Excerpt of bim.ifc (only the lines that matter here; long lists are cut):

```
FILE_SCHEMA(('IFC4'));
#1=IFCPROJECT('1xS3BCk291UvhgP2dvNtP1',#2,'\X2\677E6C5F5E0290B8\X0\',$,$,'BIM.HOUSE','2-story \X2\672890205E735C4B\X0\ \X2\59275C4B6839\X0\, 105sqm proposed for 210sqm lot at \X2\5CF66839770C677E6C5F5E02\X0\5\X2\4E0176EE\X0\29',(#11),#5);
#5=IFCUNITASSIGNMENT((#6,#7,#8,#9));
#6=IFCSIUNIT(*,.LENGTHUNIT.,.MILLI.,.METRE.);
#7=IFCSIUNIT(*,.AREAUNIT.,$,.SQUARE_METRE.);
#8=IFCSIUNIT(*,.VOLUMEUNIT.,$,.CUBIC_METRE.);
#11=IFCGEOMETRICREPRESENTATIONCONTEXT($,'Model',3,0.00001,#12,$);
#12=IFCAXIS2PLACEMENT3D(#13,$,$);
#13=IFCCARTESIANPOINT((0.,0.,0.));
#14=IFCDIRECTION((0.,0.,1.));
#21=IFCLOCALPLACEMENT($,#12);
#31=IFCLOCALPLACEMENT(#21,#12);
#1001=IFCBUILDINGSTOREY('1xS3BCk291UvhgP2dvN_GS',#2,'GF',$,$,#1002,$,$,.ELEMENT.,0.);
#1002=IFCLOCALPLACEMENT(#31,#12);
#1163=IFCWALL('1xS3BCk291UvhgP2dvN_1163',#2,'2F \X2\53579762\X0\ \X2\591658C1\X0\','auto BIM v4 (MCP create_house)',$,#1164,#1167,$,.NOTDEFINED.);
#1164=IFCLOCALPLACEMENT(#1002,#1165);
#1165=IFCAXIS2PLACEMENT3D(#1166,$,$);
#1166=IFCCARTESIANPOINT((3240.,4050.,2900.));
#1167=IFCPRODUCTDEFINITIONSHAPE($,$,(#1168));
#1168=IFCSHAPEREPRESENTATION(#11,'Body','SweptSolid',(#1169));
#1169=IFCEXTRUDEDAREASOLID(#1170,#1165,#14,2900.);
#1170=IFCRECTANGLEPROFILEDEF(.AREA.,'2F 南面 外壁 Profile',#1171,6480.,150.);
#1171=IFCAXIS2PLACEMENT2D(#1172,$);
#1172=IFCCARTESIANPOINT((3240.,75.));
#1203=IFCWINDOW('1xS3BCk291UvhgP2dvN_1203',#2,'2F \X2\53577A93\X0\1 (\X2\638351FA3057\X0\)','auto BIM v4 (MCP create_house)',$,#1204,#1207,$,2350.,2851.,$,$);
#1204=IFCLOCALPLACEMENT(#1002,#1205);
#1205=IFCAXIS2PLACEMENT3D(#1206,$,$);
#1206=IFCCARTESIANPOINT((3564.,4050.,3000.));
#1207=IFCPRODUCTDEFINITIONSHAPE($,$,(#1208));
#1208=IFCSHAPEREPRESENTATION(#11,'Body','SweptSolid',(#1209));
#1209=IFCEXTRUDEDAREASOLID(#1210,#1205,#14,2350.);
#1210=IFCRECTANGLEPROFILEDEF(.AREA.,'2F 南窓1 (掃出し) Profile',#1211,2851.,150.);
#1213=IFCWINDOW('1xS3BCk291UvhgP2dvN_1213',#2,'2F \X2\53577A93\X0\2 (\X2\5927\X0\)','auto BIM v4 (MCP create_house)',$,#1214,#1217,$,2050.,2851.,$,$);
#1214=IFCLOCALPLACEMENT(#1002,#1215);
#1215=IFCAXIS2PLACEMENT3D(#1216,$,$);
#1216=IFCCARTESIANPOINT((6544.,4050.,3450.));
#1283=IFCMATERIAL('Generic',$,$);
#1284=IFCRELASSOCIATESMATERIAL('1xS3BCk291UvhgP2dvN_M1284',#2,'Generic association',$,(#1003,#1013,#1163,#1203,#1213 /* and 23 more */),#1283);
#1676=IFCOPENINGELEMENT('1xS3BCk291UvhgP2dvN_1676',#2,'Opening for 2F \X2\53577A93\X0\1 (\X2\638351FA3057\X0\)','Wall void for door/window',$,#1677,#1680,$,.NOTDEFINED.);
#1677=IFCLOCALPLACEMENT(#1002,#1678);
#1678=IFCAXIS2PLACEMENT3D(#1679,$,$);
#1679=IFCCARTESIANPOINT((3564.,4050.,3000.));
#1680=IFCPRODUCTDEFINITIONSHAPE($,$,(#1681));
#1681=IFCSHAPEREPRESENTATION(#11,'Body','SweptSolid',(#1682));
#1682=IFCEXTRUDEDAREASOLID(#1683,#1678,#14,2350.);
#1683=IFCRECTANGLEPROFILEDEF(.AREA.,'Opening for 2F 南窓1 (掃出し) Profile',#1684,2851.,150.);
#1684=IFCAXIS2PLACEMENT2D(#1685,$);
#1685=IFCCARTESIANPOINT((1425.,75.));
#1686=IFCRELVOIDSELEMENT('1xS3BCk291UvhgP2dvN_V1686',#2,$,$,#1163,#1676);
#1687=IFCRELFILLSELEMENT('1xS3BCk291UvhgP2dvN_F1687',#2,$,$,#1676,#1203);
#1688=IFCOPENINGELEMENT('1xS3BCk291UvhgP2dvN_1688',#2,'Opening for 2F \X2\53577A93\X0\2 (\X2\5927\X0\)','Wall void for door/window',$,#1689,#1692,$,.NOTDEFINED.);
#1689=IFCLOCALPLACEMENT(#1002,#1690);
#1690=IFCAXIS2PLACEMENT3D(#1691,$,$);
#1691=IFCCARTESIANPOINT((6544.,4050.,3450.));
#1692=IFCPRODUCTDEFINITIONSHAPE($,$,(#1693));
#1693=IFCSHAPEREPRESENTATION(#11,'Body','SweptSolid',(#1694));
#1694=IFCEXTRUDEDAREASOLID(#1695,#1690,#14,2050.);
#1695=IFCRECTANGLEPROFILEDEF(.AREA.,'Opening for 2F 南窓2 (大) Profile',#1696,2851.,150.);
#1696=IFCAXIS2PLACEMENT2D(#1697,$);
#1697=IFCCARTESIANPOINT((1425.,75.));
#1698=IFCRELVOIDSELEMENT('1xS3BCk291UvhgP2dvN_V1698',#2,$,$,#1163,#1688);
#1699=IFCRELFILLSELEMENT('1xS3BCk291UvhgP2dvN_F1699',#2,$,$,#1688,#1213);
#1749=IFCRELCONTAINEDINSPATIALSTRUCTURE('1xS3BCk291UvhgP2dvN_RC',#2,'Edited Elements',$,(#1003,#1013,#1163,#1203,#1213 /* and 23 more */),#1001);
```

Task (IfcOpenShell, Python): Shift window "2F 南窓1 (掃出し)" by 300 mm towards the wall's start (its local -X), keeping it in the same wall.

```python
import ifcopenshell
import ifcopenshell.api.geometry
import ifcopenshell.util.placement
import ifcopenshell.util.unit

model = ifcopenshell.open("bim.ifc")
unit_scale = ifcopenshell.util.unit.calculate_unit_scale(model)

window = model.by_id(1203)
opening = window.FillsVoids[0].RelatingOpeningElement
wall = opening.VoidsElements[0].RelatingBuildingElement

wall_matrix = ifcopenshell.util.placement.get_local_placement(wall.ObjectPlacement)
shift = wall_matrix[:3, 0] * -0.3 / unit_scale
before = ifcopenshell.util.placement.get_local_placement(window.ObjectPlacement)[:3, 3].copy()

# The window is not placed relative to its opening, so move both.
for product in (opening, window):
    matrix = ifcopenshell.util.placement.get_local_placement(product.ObjectPlacement)
    matrix[:3, 3] += shift
    ifcopenshell.api.geometry.edit_object_placement(model, product=product, matrix=matrix, is_si=False)

after = ifcopenshell.util.placement.get_local_placement(window.ObjectPlacement)[:3, 3]
print("window moved by", (after - before).round(3) + 0.0)

model.write("bim_updated.ifc")
```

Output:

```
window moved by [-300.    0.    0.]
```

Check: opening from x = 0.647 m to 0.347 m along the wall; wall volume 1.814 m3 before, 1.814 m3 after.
